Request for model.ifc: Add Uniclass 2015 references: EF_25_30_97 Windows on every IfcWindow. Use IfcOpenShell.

First a look at what the model holds.

```python
import ifcopenshell

model = ifcopenshell.open("model.ifc")
print(model.schema)
print("classifications:", [c.Name for c in model.by_type("IfcClassification")])
for ifc_class in ("IfcDoor", "IfcRoof", "IfcStair", "IfcWall", "IfcWindow"):
    print(ifc_class, len(model.by_type(ifc_class)))
```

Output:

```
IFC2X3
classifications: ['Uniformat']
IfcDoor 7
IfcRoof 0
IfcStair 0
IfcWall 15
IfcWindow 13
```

```python
import ifcopenshell
import ifcopenshell.api.classification

model = ifcopenshell.open("model.ifc")

# IFC2X3 requires Source and Edition and has no link from the project to the system.
system = model.create_entity("IfcClassification", Source="NBS", Edition="2015", Name="Uniclass 2015")

codes = {
    "IfcWindow": ("EF_25_30_97", "Windows"),
}
for ifc_class, (code, name) in codes.items():
    products = model.by_type(ifc_class)
    ifcopenshell.api.classification.add_reference(
        model, products=products, classification=system, identification=code, name=name
    )
    print(code, len(products))

model.write("model-out.ifc")
```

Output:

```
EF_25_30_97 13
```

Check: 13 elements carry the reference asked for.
